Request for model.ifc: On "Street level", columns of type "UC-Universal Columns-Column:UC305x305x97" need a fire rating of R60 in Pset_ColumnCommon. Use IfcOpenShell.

First a look at what the model holds.

```python
import ifcopenshell
import ifcopenshell.util.element

model = ifcopenshell.open("model.ifc")
print(model.schema)
storey = next(s for s in model.by_type("IfcBuildingStorey") if s.Name == "Street level")
columns = [e for e in ifcopenshell.util.element.get_decomposition(storey) if e.is_a("IfcColumn")]
seen = {}
for e in columns:
    element_type = ifcopenshell.util.element.get_type(e)
    key = (element_type.Name if element_type != e and element_type else None, ifcopenshell.util.element.get_pset(e, "Pset_ColumnCommon", "FireRating"))
    seen[key] = seen.get(key, 0) + 1
for (name, value), count in sorted(seen.items(), key=str):
    print(count, "x", name, "|", value)
```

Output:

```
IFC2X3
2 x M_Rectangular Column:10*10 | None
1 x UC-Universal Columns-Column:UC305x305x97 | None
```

```python
import ifcopenshell
import ifcopenshell.api.pset
import ifcopenshell.util.element

model = ifcopenshell.open("model.ifc")

storey = next(s for s in model.by_type("IfcBuildingStorey") if s.Name == "Street level")
columns = [e for e in ifcopenshell.util.element.get_decomposition(storey) if e.is_a("IfcColumn")]

count = 0
for e in columns:
    element_type = ifcopenshell.util.element.get_type(e)
    if element_type in (None, e) or element_type.Name != "UC-Universal Columns-Column:UC305x305x97":
        continue
    # add_pset returns the element's existing set when there is one.
    pset = ifcopenshell.api.pset.add_pset(model, product=e, name="Pset_ColumnCommon")
    ifcopenshell.api.pset.edit_pset(model, pset=pset, properties={"FireRating": "R60"})
    count += 1

print(count, "columns updated")

model.write("model_rev.ifc")
```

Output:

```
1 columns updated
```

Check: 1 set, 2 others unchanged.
